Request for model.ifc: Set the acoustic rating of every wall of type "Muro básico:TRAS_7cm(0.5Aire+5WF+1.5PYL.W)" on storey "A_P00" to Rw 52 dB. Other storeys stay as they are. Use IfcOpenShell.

First a look at what the model holds.

```python
import ifcopenshell
import ifcopenshell.util.element

model = ifcopenshell.open("model.ifc")
print(model.schema)
storey = next(s for s in model.by_type("IfcBuildingStorey") if s.Name == "A_P00")
walls = [e for e in ifcopenshell.util.element.get_decomposition(storey) if e.is_a("IfcWall")]
seen = {}
for e in walls:
    element_type = ifcopenshell.util.element.get_type(e)
    key = (element_type.Name if element_type != e and element_type else None, ifcopenshell.util.element.get_pset(e, "Pset_WallCommon", "AcousticRating"))
    seen[key] = seen.get(key, 0) + 1
for (name, value), count in sorted(seen.items(), key=str):
    print(count, "x", name, "|", value)
```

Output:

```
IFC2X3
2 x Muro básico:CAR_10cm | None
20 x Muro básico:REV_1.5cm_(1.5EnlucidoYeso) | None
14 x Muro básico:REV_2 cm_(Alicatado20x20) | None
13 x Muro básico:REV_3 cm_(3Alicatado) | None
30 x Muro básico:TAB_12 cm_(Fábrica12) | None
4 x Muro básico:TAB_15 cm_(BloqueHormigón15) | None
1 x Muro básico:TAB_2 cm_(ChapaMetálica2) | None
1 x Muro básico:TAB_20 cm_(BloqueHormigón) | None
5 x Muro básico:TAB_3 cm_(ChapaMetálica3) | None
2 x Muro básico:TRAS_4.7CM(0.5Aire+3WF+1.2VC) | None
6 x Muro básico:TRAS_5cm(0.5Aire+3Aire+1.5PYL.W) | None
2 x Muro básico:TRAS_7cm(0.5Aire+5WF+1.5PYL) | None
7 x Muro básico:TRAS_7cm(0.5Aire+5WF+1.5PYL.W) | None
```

```python
import ifcopenshell
import ifcopenshell.api.pset
import ifcopenshell.util.element

model = ifcopenshell.open("model.ifc")

storey = next(s for s in model.by_type("IfcBuildingStorey") if s.Name == "A_P00")
walls = [e for e in ifcopenshell.util.element.get_decomposition(storey) if e.is_a("IfcWall")]

count = 0
for e in walls:
    element_type = ifcopenshell.util.element.get_type(e)
    if element_type in (None, e) or element_type.Name != "Muro básico:TRAS_7cm(0.5Aire+5WF+1.5PYL.W)":
        continue
    # add_pset returns the element's existing set when there is one.
    pset = ifcopenshell.api.pset.add_pset(model, product=e, name="Pset_WallCommon")
    ifcopenshell.api.pset.edit_pset(model, pset=pset, properties={"AcousticRating": "Rw 52 dB"})
    count += 1

print(count, "walls updated")

model.write("model_updated.ifc")
```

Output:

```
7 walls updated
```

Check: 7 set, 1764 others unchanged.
